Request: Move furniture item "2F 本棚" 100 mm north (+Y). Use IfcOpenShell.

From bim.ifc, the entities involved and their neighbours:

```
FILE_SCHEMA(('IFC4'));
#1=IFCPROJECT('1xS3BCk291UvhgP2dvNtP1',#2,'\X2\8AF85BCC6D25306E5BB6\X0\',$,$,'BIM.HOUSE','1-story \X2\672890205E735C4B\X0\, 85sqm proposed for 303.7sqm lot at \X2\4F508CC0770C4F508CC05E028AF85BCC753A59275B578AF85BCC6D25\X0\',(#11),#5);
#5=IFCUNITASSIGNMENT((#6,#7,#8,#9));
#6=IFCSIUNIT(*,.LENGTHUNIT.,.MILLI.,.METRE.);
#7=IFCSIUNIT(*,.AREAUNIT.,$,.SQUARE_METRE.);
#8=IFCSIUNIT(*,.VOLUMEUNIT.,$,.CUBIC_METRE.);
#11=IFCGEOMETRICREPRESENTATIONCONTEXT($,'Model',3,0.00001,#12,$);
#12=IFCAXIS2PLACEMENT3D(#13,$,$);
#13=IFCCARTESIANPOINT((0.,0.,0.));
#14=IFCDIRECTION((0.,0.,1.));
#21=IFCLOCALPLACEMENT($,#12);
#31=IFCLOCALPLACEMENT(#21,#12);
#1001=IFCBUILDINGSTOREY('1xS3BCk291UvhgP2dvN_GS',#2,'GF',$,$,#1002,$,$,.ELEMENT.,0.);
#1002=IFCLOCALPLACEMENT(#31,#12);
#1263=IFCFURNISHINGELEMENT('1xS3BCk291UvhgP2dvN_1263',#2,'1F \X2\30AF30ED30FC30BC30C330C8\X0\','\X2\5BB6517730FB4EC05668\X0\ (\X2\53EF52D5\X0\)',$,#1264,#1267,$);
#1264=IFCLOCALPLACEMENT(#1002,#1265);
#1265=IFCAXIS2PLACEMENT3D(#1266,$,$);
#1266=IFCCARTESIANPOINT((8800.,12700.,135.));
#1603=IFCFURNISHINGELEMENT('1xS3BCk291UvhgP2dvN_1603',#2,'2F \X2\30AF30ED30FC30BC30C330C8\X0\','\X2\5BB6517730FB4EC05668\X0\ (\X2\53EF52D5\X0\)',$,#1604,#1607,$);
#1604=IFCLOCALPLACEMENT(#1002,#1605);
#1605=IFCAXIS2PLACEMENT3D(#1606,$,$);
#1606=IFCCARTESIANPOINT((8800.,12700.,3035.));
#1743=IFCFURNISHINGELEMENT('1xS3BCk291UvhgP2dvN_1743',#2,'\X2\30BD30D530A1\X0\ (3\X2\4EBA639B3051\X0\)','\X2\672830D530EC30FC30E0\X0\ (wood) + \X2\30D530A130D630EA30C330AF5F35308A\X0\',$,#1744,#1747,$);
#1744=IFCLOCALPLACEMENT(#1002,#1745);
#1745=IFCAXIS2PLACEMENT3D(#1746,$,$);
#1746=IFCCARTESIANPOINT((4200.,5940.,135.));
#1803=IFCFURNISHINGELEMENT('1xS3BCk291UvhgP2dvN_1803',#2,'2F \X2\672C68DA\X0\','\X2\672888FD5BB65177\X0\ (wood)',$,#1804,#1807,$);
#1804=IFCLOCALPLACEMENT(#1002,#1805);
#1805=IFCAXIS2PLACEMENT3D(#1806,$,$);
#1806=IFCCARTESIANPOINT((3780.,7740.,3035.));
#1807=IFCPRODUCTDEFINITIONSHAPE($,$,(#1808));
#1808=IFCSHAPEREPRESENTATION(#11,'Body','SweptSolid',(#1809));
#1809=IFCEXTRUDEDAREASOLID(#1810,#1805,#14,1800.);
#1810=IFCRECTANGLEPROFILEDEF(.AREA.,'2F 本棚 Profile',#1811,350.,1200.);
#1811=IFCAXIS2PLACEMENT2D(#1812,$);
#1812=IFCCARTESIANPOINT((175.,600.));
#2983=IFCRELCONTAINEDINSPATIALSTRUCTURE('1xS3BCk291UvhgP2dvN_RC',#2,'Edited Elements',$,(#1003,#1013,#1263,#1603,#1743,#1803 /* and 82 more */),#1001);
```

```python
import ifcopenshell
import ifcopenshell.api.geometry
import ifcopenshell.util.placement

model = ifcopenshell.open("bim.ifc")

item = model.by_id(1803)
matrix = ifcopenshell.util.placement.get_local_placement(item.ObjectPlacement)
matrix[1, 3] += 100.0
ifcopenshell.api.geometry.edit_object_placement(model, product=item, matrix=matrix, is_si=False)

print(ifcopenshell.util.placement.get_local_placement(item.ObjectPlacement).round(3) + 0.0)

model.write("bim_rev.ifc")
```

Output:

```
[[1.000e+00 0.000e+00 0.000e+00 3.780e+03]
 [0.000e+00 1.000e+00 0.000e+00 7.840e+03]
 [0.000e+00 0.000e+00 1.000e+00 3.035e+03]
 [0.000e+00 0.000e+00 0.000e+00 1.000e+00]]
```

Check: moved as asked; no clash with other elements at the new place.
